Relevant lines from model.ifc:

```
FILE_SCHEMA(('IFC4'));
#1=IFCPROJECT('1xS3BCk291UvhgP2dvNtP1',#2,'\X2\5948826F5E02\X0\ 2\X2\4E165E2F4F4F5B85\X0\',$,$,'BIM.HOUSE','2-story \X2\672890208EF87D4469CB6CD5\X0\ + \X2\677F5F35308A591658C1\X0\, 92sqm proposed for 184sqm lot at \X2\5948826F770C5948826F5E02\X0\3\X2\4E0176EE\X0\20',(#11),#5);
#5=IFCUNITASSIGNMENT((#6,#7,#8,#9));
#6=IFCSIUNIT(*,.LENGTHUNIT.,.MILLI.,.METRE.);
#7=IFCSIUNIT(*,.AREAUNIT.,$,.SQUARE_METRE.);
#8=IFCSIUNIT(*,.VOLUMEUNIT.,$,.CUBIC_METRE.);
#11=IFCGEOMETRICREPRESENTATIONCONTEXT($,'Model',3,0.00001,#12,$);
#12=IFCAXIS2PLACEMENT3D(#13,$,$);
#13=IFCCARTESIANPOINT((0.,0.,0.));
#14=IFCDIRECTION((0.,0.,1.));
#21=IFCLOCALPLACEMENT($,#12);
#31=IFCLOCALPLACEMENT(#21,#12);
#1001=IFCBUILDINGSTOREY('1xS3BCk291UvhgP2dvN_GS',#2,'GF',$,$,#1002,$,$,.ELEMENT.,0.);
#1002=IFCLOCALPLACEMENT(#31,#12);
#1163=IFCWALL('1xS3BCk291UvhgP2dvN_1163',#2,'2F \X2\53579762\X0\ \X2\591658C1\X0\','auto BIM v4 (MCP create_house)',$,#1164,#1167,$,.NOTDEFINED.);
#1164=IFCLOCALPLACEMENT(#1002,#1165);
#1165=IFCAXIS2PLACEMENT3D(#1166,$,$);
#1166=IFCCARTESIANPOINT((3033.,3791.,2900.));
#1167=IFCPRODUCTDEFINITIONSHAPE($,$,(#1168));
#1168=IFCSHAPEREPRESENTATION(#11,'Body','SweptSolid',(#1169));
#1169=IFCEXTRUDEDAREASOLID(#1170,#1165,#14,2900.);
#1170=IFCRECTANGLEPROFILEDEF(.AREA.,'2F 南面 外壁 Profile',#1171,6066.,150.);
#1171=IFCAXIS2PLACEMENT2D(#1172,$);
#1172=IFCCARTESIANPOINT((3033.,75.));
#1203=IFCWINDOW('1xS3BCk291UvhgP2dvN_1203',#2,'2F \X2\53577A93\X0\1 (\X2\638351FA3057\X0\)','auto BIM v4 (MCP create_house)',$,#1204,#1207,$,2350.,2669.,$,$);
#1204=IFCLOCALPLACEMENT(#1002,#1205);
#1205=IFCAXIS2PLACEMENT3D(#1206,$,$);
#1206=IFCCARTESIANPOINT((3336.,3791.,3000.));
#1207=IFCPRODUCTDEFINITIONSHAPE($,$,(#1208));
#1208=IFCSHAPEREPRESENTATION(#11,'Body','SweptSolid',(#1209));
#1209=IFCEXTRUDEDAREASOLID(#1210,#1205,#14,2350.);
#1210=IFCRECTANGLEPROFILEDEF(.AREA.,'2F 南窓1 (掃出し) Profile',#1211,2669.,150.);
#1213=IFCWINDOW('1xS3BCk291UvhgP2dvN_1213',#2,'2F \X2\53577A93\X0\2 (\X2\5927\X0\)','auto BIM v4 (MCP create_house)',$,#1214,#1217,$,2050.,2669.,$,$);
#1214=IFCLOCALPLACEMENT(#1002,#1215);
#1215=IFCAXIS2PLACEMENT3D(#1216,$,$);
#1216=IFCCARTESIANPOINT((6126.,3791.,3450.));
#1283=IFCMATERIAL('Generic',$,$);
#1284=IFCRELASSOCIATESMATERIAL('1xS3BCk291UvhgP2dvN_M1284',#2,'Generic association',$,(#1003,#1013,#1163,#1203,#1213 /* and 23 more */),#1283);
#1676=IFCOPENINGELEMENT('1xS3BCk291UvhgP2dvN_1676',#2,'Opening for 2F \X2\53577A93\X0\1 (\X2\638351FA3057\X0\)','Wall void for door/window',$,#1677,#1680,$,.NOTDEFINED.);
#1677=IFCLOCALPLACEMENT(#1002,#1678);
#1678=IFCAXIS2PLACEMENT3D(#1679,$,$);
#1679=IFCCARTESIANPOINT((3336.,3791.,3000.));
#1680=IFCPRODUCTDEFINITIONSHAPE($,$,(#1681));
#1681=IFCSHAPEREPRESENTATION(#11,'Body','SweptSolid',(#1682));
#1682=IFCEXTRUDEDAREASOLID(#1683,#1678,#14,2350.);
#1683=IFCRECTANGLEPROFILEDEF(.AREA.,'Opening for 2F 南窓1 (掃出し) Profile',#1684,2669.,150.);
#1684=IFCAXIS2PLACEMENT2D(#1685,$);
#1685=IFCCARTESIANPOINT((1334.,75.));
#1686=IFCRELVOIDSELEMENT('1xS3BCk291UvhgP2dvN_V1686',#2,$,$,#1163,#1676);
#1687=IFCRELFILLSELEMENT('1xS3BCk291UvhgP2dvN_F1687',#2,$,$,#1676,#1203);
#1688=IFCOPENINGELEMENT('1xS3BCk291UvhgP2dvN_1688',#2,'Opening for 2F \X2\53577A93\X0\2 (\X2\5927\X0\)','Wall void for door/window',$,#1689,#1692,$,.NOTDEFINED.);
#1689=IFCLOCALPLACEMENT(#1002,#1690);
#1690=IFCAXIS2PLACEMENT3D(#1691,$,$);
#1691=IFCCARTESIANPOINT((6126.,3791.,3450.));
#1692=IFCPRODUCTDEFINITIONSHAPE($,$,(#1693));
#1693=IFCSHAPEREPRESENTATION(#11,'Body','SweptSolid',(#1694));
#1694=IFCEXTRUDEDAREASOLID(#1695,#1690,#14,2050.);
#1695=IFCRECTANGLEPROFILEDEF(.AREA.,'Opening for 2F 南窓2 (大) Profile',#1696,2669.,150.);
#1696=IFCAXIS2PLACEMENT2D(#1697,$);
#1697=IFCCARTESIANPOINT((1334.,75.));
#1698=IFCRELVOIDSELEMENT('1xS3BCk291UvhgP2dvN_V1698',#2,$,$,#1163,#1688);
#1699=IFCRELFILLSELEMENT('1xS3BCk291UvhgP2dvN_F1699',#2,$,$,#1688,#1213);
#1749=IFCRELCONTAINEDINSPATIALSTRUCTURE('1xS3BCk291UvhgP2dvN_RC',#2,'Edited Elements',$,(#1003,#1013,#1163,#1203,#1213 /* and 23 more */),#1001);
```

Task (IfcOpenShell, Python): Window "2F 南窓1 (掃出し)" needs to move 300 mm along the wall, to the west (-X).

```python
import ifcopenshell
import ifcopenshell.api.geometry
import ifcopenshell.util.placement
import ifcopenshell.util.unit

model = ifcopenshell.open("model.ifc")
unit_scale = ifcopenshell.util.unit.calculate_unit_scale(model)

window = model.by_guid("1xS3BCk291UvhgP2dvN_1203")
opening = window.FillsVoids[0].RelatingOpeningElement
wall = opening.VoidsElements[0].RelatingBuildingElement

wall_matrix = ifcopenshell.util.placement.get_local_placement(wall.ObjectPlacement)
shift = wall_matrix[:3, 0] * -0.3 / unit_scale
before = ifcopenshell.util.placement.get_local_placement(window.ObjectPlacement)[:3, 3].copy()

# The window is not placed relative to its opening, so move both.
for product in (opening, window):
    matrix = ifcopenshell.util.placement.get_local_placement(product.ObjectPlacement)
    matrix[:3, 3] += shift
    ifcopenshell.api.geometry.edit_object_placement(model, product=product, matrix=matrix, is_si=False)

after = ifcopenshell.util.placement.get_local_placement(window.ObjectPlacement)[:3, 3]
print("window moved by", (after - before).round(3) + 0.0)

model.write("model_rev.ifc")
```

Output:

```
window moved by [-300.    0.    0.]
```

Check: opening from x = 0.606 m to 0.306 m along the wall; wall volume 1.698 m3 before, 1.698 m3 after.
